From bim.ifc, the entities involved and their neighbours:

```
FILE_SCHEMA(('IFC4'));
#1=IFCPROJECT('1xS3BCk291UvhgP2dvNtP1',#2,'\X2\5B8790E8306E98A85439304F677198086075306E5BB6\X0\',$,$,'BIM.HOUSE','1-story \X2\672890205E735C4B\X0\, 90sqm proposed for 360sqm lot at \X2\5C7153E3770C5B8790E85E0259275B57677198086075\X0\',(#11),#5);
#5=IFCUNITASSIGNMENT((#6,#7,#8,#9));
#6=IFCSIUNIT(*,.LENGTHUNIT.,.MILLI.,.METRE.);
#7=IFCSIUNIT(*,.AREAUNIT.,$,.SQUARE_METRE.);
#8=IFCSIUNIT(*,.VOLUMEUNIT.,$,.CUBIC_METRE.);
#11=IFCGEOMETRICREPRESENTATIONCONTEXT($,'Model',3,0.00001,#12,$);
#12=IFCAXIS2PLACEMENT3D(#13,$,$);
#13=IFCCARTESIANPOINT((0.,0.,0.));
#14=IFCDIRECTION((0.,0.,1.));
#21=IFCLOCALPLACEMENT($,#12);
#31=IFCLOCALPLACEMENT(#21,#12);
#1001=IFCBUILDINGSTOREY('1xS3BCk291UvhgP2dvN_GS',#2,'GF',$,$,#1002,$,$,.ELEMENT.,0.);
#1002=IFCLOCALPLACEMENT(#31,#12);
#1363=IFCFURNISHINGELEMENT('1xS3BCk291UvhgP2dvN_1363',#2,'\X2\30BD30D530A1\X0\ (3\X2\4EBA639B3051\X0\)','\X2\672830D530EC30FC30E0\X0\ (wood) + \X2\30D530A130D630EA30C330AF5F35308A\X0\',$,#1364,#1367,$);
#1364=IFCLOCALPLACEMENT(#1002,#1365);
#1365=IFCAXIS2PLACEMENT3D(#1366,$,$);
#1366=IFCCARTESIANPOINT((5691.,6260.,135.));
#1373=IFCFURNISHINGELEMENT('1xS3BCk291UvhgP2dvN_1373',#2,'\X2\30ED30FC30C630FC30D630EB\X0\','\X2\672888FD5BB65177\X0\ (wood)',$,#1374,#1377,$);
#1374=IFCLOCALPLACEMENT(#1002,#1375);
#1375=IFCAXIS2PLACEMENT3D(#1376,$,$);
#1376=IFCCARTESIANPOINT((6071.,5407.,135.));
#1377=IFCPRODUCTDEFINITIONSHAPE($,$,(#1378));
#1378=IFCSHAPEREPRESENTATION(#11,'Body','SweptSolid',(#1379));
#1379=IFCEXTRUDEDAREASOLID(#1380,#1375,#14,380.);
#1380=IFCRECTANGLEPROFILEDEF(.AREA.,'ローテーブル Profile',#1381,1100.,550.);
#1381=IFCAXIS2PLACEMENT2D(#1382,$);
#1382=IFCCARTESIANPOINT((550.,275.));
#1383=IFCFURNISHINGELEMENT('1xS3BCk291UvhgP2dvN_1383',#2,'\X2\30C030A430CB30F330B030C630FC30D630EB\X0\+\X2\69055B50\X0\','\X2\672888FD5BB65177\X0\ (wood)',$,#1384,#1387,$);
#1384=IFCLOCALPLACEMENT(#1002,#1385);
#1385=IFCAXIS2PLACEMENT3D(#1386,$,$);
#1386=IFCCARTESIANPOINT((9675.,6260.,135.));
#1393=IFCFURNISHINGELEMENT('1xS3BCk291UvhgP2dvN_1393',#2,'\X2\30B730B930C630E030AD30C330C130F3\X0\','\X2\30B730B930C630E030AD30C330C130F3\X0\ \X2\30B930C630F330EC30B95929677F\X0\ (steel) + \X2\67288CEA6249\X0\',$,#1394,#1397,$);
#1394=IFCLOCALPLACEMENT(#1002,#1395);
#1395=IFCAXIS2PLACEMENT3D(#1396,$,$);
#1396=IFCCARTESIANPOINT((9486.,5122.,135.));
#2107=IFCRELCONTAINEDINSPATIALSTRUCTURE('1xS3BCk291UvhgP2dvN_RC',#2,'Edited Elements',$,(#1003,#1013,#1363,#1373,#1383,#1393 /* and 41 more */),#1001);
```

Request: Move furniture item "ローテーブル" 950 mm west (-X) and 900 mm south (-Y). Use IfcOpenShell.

```python
import ifcopenshell
import ifcopenshell.api.geometry
import ifcopenshell.util.placement

model = ifcopenshell.open("bim.ifc")

item = model.by_guid("1xS3BCk291UvhgP2dvN_1373")
matrix = ifcopenshell.util.placement.get_local_placement(item.ObjectPlacement)
matrix[0, 3] -= 950.0
matrix[1, 3] -= 900.0
ifcopenshell.api.geometry.edit_object_placement(model, product=item, matrix=matrix, is_si=False)

print(ifcopenshell.util.placement.get_local_placement(item.ObjectPlacement).round(3) + 0.0)

model.write("bim_v2.ifc")
```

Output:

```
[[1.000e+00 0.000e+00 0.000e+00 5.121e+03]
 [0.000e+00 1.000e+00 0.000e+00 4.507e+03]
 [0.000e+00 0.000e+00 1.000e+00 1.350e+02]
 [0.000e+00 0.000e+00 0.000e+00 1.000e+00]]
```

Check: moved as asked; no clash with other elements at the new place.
